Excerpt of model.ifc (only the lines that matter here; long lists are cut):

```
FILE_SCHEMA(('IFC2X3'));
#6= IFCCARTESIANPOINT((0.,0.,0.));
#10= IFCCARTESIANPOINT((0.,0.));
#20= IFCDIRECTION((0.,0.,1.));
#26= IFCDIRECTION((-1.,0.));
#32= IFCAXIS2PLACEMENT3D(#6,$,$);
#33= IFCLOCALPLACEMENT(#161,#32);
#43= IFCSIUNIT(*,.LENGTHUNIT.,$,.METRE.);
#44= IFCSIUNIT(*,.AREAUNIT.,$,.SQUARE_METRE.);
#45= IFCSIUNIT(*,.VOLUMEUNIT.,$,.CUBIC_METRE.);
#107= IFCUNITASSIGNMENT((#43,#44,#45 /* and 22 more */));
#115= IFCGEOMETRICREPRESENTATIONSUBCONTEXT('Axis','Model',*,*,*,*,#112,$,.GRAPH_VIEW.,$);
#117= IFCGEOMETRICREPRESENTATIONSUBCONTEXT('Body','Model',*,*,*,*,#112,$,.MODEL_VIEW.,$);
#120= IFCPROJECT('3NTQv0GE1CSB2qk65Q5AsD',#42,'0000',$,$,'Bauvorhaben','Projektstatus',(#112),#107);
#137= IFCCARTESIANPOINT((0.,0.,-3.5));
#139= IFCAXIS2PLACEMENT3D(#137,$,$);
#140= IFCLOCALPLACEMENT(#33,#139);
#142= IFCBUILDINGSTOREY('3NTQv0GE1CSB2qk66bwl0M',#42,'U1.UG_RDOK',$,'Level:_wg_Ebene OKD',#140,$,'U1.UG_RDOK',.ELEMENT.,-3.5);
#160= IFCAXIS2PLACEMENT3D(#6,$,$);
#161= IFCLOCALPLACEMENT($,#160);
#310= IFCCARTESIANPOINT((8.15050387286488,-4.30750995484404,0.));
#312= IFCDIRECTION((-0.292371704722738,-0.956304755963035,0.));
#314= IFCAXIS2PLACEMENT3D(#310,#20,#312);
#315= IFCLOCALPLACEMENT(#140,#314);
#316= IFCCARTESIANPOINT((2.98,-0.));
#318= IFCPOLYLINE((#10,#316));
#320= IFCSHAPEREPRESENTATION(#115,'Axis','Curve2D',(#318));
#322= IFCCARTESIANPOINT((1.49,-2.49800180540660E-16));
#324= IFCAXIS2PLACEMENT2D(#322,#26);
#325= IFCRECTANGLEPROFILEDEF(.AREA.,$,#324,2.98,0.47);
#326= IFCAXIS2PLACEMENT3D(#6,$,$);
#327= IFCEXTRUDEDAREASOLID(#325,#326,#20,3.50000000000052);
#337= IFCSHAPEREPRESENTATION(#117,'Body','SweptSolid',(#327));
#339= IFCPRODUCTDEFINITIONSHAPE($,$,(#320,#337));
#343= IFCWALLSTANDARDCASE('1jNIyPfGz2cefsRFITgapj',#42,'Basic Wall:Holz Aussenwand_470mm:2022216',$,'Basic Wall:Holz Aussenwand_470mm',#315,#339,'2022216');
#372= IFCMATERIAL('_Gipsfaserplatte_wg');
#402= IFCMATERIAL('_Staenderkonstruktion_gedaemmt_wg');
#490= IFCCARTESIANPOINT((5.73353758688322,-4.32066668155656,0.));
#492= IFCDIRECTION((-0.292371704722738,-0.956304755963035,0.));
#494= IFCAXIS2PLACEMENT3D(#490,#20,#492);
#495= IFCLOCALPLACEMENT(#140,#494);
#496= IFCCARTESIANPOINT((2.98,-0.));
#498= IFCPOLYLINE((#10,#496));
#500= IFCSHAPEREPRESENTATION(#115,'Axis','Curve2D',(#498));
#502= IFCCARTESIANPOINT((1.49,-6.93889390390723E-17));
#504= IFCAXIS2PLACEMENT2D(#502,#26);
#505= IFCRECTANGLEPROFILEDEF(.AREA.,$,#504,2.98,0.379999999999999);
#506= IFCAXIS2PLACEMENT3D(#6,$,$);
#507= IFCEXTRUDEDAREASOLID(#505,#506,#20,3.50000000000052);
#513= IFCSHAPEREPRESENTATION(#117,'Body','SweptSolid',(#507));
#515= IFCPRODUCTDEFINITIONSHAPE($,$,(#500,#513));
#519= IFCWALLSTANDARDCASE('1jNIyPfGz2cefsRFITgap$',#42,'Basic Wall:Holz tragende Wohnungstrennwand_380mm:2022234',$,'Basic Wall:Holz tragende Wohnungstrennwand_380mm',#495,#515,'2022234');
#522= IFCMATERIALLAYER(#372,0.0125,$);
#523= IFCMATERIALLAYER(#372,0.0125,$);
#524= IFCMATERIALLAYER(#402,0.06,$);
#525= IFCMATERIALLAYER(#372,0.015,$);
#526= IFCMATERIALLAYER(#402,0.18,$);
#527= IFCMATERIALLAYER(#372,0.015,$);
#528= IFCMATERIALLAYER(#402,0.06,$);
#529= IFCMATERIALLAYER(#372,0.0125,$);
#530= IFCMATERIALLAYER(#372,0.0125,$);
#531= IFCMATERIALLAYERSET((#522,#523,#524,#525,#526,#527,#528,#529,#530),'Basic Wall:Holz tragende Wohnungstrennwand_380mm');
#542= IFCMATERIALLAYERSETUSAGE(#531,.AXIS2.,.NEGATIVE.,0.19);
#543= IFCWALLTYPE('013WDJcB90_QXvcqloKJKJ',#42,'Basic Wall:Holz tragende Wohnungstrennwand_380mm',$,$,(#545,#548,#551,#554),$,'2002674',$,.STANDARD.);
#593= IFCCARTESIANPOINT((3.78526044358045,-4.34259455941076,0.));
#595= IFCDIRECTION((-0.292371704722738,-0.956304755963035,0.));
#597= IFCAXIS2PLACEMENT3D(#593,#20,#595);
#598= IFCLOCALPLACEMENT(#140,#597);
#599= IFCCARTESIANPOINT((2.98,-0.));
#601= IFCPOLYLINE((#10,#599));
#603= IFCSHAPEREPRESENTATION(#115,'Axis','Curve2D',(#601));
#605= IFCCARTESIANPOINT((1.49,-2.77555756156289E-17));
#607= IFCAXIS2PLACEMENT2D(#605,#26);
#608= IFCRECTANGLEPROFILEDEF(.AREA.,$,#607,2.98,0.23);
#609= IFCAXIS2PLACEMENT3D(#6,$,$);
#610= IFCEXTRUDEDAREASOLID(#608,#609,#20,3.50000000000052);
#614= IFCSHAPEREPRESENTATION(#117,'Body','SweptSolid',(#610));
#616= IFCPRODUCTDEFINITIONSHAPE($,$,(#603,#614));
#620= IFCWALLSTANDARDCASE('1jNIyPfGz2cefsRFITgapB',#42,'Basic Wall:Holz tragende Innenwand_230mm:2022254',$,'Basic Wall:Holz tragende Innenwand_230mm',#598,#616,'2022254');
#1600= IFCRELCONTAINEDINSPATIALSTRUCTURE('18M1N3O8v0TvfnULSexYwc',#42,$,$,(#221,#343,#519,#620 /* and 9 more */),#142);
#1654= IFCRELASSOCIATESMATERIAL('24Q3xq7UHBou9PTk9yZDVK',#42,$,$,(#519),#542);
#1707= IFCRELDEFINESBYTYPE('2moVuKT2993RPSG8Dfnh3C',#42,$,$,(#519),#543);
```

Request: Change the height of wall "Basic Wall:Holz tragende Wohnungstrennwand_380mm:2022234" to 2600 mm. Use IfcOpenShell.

```python
import ifcopenshell
import ifcopenshell.geom
import ifcopenshell.util.representation
import ifcopenshell.util.shape
import ifcopenshell.util.unit

model = ifcopenshell.open("model.ifc")
unit_scale = ifcopenshell.util.unit.calculate_unit_scale(model)
settings = ifcopenshell.geom.settings()


def volume(element):
    """Net volume in cubic metres, openings subtracted."""
    shape = ifcopenshell.geom.create_shape(settings, element)
    return ifcopenshell.util.shape.get_volume(shape.geometry)


wall = model.by_guid("1jNIyPfGz2cefsRFITgap$")
before = volume(wall)

body = ifcopenshell.util.representation.get_representation(wall, "Model", "Body")
solid = body.Items[0]
old_height = solid.Depth
solid.Depth = 2.6 / unit_scale
after = volume(wall)

print(f"height {old_height:g} -> {solid.Depth:g}, volume {before:.3f} -> {after:.3f} m3")

model.write("model_v2.ifc")
```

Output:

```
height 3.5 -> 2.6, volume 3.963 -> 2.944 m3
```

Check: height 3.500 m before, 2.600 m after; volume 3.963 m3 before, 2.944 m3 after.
